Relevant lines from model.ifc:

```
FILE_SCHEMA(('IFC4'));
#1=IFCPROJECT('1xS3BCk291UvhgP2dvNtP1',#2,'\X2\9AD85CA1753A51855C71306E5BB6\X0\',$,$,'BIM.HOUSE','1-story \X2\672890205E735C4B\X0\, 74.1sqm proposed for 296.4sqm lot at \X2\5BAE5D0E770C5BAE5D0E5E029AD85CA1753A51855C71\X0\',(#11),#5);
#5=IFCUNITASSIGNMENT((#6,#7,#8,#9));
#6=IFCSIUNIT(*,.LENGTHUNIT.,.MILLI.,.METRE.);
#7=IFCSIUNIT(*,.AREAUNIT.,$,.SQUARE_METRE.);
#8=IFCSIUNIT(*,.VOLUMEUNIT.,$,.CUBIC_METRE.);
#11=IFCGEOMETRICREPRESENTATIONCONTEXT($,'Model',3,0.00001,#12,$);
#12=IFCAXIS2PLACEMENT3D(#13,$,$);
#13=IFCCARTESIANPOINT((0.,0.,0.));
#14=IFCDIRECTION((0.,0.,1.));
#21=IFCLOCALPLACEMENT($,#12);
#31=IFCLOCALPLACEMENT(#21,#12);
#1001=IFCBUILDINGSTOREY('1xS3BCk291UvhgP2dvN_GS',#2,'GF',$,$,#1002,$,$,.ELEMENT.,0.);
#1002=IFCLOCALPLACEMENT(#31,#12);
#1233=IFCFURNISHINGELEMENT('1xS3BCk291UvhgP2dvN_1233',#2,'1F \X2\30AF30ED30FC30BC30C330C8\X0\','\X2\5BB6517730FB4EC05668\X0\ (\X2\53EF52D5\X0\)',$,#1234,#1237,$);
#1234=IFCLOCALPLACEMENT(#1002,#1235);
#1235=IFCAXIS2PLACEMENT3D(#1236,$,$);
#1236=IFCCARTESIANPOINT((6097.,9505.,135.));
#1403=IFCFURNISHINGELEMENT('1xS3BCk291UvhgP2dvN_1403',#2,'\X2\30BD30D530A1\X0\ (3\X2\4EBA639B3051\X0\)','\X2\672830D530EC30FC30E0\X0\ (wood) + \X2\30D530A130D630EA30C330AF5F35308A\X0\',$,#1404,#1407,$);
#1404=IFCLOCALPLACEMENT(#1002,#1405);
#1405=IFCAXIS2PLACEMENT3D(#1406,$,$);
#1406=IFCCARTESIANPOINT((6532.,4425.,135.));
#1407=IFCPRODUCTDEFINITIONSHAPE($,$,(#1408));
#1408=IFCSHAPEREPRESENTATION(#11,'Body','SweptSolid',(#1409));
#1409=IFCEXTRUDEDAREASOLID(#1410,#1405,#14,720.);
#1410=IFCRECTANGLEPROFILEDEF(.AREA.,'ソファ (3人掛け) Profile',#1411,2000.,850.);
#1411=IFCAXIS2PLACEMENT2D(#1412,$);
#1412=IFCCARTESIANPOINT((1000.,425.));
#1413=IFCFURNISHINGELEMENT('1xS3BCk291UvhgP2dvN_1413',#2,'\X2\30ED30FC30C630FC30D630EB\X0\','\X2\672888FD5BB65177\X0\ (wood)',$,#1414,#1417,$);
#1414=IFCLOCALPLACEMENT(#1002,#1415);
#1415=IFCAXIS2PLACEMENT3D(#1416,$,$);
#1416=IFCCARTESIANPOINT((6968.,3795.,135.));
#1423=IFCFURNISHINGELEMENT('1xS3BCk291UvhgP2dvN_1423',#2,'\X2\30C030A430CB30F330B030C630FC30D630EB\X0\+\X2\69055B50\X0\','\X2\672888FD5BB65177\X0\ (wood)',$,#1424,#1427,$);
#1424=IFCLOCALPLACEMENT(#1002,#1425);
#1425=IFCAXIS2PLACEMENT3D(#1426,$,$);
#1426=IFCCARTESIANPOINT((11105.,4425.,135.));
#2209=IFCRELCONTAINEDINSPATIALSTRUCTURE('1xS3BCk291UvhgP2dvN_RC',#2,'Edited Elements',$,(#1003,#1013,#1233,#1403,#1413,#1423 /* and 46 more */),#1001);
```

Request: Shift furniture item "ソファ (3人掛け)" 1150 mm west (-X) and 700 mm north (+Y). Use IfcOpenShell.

```python
import ifcopenshell
import ifcopenshell.api.geometry
import ifcopenshell.util.placement

model = ifcopenshell.open("model.ifc")

item = model.by_guid("1xS3BCk291UvhgP2dvN_1403")
matrix = ifcopenshell.util.placement.get_local_placement(item.ObjectPlacement)
matrix[0, 3] -= 1150.0
matrix[1, 3] += 700.0
ifcopenshell.api.geometry.edit_object_placement(model, product=item, matrix=matrix, is_si=False)

print(ifcopenshell.util.placement.get_local_placement(item.ObjectPlacement).round(3) + 0.0)

model.write("model_v2.ifc")
```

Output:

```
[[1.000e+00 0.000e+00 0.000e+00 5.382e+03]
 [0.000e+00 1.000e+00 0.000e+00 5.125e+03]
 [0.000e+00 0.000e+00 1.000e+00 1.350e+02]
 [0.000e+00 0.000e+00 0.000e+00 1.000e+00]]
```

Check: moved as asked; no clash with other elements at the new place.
